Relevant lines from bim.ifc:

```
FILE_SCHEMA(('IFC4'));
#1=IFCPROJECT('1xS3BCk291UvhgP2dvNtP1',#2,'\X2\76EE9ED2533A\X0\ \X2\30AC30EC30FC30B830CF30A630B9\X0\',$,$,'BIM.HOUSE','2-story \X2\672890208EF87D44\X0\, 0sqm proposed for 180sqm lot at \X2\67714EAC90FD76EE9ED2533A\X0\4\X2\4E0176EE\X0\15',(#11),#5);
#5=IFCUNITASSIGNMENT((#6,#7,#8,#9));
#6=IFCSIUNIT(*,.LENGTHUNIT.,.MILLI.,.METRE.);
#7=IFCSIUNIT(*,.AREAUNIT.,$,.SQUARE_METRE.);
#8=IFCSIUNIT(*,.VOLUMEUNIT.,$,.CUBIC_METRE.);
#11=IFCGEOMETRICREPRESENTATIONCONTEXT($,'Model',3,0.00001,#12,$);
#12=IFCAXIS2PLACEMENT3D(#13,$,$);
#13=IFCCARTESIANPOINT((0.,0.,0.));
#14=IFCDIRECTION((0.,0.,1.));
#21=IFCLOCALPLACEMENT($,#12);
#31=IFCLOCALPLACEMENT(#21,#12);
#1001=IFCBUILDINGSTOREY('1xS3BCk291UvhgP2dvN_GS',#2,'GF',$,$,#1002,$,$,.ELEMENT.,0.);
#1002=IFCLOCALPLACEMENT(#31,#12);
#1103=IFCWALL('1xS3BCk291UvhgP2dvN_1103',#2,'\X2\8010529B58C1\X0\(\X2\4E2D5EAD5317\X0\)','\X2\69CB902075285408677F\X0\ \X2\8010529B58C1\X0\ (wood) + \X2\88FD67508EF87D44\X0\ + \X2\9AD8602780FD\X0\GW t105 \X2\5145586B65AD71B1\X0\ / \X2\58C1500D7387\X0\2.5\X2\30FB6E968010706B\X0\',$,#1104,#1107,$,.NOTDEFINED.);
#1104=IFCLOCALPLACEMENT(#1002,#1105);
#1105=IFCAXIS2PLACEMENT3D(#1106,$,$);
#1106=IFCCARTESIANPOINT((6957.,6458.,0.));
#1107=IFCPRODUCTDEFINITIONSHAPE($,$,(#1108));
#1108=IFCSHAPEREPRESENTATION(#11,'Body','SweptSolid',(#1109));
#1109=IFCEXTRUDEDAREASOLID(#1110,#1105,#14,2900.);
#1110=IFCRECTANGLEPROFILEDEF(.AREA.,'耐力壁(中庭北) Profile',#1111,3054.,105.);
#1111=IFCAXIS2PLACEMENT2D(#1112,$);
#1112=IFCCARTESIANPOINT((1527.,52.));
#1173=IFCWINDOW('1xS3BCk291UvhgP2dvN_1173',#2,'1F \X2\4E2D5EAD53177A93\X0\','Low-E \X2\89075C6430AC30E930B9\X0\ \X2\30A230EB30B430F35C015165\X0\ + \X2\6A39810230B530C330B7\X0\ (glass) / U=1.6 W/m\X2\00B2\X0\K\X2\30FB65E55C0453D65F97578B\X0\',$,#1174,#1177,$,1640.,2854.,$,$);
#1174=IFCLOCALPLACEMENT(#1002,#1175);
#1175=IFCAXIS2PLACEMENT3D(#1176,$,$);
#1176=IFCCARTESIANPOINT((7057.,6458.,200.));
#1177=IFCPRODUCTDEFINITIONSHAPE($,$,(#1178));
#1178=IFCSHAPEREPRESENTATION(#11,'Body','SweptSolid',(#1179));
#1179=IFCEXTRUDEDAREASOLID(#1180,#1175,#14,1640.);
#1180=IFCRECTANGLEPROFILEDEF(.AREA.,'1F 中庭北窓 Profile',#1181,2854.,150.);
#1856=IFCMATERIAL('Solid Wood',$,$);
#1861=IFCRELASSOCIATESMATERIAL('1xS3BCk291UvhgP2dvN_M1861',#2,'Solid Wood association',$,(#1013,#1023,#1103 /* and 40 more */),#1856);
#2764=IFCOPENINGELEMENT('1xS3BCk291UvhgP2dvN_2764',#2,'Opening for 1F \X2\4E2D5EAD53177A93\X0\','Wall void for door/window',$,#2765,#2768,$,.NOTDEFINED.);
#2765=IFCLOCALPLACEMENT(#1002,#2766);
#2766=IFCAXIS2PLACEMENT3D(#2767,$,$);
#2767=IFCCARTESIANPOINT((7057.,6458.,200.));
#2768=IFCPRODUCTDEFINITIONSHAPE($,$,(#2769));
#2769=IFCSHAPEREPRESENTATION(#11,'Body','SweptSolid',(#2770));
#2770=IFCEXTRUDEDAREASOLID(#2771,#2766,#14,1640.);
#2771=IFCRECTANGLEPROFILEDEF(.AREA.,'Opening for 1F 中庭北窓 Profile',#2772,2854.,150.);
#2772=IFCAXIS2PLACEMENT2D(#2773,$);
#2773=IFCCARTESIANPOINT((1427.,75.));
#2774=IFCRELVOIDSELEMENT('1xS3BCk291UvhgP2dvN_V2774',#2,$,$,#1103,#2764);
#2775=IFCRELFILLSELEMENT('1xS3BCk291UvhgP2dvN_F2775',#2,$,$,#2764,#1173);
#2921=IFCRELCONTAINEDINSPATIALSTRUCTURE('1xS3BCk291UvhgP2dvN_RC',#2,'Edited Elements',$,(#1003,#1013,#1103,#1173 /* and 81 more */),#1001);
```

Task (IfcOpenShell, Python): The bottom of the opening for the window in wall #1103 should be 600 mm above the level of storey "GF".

```python
import numpy as np
import ifcopenshell
import ifcopenshell.api.geometry
import ifcopenshell.geom
import ifcopenshell.util.element
import ifcopenshell.util.placement
import ifcopenshell.util.shape
import ifcopenshell.util.unit

model = ifcopenshell.open("bim.ifc")
unit_scale = ifcopenshell.util.unit.calculate_unit_scale(model)

window = model.by_guid("1xS3BCk291UvhgP2dvN_1173")
opening = window.FillsVoids[0].RelatingOpeningElement
storey = ifcopenshell.util.element.get_container(window, ifc_class="IfcBuildingStorey")
level = ifcopenshell.util.placement.get_local_placement(storey.ObjectPlacement)[2, 3]

# The opening's origin need not be at the sill, so measure its lowest point.
shape = ifcopenshell.geom.create_shape(ifcopenshell.geom.settings(), opening)
bottom = ifcopenshell.util.shape.get_shape_bottom_elevation(shape, shape.geometry) / unit_scale
dz = level + 600.0 - bottom

shift = np.array([0.0, 0.0, dz])
# The window is not placed relative to its opening, so move both.
for product in (opening, window):
    matrix = ifcopenshell.util.placement.get_local_placement(product.ObjectPlacement)
    matrix[:3, 3] += shift
    ifcopenshell.api.geometry.edit_object_placement(model, product=product, matrix=matrix, is_si=False)

print(f"moved by {dz * unit_scale:+.3f} m")

model.write("bim_edited.ifc")
```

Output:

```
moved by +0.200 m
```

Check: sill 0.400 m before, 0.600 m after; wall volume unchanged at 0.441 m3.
